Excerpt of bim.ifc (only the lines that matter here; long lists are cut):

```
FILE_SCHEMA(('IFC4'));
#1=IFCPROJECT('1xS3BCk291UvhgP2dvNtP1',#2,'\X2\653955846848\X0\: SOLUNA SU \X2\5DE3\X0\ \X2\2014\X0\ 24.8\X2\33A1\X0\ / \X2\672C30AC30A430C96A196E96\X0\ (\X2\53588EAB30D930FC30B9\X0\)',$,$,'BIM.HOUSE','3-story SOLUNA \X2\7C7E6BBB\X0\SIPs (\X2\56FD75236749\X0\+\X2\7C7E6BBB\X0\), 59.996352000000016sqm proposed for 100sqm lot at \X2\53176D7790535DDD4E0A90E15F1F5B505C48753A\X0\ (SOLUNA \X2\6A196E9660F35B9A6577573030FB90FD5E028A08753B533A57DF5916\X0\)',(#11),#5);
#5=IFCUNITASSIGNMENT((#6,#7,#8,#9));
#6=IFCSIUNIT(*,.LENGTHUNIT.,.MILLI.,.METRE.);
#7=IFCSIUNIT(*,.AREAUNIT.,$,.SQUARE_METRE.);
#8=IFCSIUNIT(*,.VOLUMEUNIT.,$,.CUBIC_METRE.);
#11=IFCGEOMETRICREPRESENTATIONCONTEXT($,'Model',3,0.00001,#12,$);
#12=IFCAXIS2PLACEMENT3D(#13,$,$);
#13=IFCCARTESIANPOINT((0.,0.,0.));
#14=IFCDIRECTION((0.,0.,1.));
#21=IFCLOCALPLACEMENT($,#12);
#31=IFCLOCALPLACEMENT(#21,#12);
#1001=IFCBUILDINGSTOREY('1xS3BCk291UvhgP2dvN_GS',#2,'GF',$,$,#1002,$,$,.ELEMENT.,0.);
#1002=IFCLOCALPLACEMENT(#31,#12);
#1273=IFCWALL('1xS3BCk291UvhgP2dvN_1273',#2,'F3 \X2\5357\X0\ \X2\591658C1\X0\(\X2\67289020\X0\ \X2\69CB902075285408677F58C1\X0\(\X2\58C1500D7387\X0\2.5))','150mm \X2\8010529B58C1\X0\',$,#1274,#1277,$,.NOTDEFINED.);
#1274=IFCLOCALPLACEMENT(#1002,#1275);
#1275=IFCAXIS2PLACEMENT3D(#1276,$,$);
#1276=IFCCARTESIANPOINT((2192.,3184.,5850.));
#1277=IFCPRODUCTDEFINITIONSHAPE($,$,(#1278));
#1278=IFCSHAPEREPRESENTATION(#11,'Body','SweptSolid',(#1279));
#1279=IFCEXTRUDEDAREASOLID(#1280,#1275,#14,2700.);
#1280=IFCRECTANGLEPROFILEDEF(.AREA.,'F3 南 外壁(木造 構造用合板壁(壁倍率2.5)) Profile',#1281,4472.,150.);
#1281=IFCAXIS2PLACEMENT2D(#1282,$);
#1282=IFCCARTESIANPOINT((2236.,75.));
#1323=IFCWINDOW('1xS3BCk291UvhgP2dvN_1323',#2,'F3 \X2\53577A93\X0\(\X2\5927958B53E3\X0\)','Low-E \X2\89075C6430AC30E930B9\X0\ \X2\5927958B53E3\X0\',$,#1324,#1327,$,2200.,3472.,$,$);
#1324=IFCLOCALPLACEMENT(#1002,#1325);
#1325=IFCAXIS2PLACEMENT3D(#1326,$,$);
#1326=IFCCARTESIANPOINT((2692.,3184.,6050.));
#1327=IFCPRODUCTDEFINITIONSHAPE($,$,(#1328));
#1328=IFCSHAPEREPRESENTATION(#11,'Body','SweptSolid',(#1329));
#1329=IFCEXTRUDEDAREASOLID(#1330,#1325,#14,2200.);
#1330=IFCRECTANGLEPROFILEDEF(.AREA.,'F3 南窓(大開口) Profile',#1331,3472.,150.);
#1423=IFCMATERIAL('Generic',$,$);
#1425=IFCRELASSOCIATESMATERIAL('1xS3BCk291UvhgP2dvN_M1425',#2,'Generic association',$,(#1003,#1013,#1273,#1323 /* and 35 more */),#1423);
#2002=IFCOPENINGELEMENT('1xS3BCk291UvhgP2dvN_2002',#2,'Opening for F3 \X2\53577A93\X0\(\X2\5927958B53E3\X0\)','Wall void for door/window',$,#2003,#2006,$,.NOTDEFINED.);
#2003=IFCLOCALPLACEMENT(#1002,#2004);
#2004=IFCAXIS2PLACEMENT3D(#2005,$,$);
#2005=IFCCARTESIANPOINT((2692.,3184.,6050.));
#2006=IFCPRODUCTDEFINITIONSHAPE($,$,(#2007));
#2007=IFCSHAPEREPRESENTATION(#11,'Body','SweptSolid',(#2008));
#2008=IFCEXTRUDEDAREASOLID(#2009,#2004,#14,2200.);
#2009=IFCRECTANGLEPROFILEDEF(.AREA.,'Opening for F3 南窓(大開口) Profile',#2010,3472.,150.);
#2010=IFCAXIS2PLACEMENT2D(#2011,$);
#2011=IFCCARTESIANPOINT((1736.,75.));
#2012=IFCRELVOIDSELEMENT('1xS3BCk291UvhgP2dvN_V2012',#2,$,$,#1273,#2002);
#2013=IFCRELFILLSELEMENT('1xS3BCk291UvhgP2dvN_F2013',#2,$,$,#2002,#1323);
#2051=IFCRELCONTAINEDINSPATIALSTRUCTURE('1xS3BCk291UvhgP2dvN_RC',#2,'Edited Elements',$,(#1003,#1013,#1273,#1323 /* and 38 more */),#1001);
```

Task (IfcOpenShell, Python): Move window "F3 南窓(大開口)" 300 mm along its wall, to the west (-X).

```python
import ifcopenshell
import ifcopenshell.api.geometry
import ifcopenshell.util.placement
import ifcopenshell.util.unit

model = ifcopenshell.open("bim.ifc")
unit_scale = ifcopenshell.util.unit.calculate_unit_scale(model)

window = model.by_guid("1xS3BCk291UvhgP2dvN_1323")
opening = window.FillsVoids[0].RelatingOpeningElement
wall = opening.VoidsElements[0].RelatingBuildingElement

wall_matrix = ifcopenshell.util.placement.get_local_placement(wall.ObjectPlacement)
shift = wall_matrix[:3, 0] * -0.3 / unit_scale
before = ifcopenshell.util.placement.get_local_placement(window.ObjectPlacement)[:3, 3].copy()

# The window is not placed relative to its opening, so move both.
for product in (opening, window):
    matrix = ifcopenshell.util.placement.get_local_placement(product.ObjectPlacement)
    matrix[:3, 3] += shift
    ifcopenshell.api.geometry.edit_object_placement(model, product=product, matrix=matrix, is_si=False)

after = ifcopenshell.util.placement.get_local_placement(window.ObjectPlacement)[:3, 3]
print("window moved by", (after - before).round(3) + 0.0)

model.write("bim_v2.ifc")
```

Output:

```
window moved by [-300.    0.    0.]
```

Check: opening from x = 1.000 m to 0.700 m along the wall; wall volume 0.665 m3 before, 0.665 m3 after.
